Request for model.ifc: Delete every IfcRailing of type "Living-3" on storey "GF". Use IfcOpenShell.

First a look at what the model holds.

```python
import ifcopenshell
import ifcopenshell.util.element

model = ifcopenshell.open("model.ifc")
print(model.schema)
storey = next(s for s in model.by_type("IfcBuildingStorey") if s.Name == "GF")
railings = [e for e in ifcopenshell.util.element.get_decomposition(storey) if e.is_a("IfcRailing")]
seen = {}
for e in railings:
    element_type = ifcopenshell.util.element.get_type(e)
    name = element_type.Name if element_type not in (None, e) else None
    seen[name] = seen.get(name, 0) + 1
for name, count in sorted(seen.items(), key=str):
    print(count, "x", name)
```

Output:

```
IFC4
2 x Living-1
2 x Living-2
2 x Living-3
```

```python
import ifcopenshell
import ifcopenshell.api.root
import ifcopenshell.util.element

model = ifcopenshell.open("model.ifc")

storey = next(s for s in model.by_type("IfcBuildingStorey") if s.Name == "GF")
railings = [e for e in ifcopenshell.util.element.get_decomposition(storey) if e.is_a("IfcRailing")]
targets = [e for e in railings if (t := ifcopenshell.util.element.get_type(e)) not in (None, e) and t.Name == "Living-3"]

for e in targets:
    ifcopenshell.api.root.remove_product(model, product=e)
print(len(targets), "removed")

model.write("model-out.ifc")
```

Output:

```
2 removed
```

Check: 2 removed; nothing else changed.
